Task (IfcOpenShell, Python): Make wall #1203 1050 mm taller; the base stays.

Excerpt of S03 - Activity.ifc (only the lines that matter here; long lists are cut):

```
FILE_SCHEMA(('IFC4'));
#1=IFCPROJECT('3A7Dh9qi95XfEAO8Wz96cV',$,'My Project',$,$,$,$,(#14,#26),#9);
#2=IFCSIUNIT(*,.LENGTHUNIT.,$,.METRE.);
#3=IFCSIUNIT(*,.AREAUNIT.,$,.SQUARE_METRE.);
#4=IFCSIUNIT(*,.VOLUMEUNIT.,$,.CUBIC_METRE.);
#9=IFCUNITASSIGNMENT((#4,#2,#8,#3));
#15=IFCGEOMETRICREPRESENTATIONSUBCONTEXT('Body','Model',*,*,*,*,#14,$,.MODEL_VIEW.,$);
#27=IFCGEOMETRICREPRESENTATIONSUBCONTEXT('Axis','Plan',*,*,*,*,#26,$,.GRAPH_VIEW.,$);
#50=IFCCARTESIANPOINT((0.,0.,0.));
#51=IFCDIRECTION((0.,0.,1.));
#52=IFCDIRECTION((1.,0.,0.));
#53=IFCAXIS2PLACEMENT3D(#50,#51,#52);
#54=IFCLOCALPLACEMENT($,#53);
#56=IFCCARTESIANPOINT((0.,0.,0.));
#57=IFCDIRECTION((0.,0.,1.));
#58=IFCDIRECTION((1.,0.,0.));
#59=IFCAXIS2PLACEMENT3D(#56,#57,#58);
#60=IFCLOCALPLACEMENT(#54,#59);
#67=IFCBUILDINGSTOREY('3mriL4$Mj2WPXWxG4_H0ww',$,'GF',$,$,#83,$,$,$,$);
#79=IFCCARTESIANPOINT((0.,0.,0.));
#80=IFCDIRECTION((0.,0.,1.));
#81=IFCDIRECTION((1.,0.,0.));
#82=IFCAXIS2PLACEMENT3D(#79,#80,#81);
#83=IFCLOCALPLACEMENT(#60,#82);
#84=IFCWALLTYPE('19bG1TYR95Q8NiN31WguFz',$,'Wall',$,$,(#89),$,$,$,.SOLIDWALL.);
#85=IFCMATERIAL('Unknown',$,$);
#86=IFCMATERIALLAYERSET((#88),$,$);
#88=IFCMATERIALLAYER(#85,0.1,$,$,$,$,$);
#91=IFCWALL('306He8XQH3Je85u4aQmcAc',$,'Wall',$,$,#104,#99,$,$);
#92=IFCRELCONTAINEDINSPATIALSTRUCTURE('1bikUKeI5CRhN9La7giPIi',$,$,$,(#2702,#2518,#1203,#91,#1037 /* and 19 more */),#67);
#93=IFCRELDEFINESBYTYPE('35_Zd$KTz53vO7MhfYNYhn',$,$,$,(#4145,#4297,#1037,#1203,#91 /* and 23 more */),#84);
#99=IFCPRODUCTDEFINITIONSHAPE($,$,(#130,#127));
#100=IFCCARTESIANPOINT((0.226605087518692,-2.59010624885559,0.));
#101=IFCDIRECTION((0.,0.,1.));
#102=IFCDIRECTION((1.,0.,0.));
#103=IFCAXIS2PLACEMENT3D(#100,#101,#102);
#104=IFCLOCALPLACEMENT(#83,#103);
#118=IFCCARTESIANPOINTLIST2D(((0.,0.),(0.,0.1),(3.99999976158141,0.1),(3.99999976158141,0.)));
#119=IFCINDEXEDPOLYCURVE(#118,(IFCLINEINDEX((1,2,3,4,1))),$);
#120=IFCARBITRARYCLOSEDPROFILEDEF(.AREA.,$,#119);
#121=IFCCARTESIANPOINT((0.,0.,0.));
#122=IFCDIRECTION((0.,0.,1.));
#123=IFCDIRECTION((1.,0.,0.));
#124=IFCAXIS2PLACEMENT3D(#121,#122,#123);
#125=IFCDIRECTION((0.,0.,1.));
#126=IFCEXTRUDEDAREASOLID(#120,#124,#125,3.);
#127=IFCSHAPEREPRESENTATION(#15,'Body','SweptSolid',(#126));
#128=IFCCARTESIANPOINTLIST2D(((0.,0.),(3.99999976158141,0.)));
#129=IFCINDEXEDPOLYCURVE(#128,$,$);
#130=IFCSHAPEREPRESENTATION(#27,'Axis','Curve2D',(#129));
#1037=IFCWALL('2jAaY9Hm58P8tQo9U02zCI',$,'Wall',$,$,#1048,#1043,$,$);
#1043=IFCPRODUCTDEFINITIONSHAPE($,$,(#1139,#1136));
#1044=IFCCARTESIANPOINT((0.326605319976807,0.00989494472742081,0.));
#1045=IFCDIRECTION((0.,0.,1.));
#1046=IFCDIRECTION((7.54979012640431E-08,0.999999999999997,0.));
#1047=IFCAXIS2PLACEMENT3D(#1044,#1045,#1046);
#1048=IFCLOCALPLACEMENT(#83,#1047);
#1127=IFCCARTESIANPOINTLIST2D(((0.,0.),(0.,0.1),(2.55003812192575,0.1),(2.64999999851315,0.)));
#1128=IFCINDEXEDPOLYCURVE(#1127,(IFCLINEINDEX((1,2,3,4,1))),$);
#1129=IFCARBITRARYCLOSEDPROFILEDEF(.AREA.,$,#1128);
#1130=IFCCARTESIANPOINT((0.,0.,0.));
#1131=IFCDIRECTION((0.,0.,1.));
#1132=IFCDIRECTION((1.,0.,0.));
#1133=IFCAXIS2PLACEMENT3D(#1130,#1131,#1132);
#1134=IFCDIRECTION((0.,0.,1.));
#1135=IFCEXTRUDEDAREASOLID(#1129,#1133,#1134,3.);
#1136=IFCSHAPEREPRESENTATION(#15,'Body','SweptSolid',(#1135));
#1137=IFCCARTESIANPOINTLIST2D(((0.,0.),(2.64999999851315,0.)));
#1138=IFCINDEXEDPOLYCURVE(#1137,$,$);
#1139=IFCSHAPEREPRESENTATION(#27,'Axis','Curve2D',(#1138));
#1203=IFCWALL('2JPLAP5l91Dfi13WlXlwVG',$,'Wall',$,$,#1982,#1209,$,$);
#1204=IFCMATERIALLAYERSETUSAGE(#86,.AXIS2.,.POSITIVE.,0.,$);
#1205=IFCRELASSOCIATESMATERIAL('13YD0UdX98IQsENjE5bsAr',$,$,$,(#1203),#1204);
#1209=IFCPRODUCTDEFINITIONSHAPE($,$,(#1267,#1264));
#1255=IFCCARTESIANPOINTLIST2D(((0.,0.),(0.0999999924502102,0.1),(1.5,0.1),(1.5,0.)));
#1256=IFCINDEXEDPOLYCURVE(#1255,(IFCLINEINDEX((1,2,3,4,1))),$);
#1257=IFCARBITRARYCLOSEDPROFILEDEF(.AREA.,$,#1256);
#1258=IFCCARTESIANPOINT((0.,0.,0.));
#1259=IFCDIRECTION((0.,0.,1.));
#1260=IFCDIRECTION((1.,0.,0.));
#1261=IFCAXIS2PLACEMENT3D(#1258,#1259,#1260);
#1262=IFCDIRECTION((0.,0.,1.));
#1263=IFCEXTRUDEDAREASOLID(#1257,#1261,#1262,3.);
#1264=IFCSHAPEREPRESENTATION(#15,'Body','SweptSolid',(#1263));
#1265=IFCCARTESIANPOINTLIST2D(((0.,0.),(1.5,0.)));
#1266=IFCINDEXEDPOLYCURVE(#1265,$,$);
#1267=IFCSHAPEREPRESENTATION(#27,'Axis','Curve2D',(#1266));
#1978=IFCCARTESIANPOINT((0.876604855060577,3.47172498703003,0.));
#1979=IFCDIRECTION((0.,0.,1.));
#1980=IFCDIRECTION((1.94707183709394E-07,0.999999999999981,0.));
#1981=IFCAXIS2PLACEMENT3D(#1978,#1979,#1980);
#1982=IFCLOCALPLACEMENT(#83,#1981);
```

```python
import ifcopenshell
import ifcopenshell.geom
import ifcopenshell.util.representation
import ifcopenshell.util.shape
import ifcopenshell.util.unit

model = ifcopenshell.open("S03 - Activity.ifc")
unit_scale = ifcopenshell.util.unit.calculate_unit_scale(model)
settings = ifcopenshell.geom.settings()


def volume(element):
    """Net volume in cubic metres, openings subtracted."""
    shape = ifcopenshell.geom.create_shape(settings, element)
    return ifcopenshell.util.shape.get_volume(shape.geometry)


wall = model.by_id(1203)
before = volume(wall)

body = ifcopenshell.util.representation.get_representation(wall, "Model", "Body")
solid = body.Items[0]
old_height = solid.Depth
solid.Depth += 1.05 / unit_scale
after = volume(wall)

print(f"height {old_height:g} -> {solid.Depth:g}, volume {before:.3f} -> {after:.3f} m3")

model.write("S03 - Activity_updated.ifc")
```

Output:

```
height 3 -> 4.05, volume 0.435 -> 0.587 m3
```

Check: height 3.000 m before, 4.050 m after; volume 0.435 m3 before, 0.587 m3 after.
